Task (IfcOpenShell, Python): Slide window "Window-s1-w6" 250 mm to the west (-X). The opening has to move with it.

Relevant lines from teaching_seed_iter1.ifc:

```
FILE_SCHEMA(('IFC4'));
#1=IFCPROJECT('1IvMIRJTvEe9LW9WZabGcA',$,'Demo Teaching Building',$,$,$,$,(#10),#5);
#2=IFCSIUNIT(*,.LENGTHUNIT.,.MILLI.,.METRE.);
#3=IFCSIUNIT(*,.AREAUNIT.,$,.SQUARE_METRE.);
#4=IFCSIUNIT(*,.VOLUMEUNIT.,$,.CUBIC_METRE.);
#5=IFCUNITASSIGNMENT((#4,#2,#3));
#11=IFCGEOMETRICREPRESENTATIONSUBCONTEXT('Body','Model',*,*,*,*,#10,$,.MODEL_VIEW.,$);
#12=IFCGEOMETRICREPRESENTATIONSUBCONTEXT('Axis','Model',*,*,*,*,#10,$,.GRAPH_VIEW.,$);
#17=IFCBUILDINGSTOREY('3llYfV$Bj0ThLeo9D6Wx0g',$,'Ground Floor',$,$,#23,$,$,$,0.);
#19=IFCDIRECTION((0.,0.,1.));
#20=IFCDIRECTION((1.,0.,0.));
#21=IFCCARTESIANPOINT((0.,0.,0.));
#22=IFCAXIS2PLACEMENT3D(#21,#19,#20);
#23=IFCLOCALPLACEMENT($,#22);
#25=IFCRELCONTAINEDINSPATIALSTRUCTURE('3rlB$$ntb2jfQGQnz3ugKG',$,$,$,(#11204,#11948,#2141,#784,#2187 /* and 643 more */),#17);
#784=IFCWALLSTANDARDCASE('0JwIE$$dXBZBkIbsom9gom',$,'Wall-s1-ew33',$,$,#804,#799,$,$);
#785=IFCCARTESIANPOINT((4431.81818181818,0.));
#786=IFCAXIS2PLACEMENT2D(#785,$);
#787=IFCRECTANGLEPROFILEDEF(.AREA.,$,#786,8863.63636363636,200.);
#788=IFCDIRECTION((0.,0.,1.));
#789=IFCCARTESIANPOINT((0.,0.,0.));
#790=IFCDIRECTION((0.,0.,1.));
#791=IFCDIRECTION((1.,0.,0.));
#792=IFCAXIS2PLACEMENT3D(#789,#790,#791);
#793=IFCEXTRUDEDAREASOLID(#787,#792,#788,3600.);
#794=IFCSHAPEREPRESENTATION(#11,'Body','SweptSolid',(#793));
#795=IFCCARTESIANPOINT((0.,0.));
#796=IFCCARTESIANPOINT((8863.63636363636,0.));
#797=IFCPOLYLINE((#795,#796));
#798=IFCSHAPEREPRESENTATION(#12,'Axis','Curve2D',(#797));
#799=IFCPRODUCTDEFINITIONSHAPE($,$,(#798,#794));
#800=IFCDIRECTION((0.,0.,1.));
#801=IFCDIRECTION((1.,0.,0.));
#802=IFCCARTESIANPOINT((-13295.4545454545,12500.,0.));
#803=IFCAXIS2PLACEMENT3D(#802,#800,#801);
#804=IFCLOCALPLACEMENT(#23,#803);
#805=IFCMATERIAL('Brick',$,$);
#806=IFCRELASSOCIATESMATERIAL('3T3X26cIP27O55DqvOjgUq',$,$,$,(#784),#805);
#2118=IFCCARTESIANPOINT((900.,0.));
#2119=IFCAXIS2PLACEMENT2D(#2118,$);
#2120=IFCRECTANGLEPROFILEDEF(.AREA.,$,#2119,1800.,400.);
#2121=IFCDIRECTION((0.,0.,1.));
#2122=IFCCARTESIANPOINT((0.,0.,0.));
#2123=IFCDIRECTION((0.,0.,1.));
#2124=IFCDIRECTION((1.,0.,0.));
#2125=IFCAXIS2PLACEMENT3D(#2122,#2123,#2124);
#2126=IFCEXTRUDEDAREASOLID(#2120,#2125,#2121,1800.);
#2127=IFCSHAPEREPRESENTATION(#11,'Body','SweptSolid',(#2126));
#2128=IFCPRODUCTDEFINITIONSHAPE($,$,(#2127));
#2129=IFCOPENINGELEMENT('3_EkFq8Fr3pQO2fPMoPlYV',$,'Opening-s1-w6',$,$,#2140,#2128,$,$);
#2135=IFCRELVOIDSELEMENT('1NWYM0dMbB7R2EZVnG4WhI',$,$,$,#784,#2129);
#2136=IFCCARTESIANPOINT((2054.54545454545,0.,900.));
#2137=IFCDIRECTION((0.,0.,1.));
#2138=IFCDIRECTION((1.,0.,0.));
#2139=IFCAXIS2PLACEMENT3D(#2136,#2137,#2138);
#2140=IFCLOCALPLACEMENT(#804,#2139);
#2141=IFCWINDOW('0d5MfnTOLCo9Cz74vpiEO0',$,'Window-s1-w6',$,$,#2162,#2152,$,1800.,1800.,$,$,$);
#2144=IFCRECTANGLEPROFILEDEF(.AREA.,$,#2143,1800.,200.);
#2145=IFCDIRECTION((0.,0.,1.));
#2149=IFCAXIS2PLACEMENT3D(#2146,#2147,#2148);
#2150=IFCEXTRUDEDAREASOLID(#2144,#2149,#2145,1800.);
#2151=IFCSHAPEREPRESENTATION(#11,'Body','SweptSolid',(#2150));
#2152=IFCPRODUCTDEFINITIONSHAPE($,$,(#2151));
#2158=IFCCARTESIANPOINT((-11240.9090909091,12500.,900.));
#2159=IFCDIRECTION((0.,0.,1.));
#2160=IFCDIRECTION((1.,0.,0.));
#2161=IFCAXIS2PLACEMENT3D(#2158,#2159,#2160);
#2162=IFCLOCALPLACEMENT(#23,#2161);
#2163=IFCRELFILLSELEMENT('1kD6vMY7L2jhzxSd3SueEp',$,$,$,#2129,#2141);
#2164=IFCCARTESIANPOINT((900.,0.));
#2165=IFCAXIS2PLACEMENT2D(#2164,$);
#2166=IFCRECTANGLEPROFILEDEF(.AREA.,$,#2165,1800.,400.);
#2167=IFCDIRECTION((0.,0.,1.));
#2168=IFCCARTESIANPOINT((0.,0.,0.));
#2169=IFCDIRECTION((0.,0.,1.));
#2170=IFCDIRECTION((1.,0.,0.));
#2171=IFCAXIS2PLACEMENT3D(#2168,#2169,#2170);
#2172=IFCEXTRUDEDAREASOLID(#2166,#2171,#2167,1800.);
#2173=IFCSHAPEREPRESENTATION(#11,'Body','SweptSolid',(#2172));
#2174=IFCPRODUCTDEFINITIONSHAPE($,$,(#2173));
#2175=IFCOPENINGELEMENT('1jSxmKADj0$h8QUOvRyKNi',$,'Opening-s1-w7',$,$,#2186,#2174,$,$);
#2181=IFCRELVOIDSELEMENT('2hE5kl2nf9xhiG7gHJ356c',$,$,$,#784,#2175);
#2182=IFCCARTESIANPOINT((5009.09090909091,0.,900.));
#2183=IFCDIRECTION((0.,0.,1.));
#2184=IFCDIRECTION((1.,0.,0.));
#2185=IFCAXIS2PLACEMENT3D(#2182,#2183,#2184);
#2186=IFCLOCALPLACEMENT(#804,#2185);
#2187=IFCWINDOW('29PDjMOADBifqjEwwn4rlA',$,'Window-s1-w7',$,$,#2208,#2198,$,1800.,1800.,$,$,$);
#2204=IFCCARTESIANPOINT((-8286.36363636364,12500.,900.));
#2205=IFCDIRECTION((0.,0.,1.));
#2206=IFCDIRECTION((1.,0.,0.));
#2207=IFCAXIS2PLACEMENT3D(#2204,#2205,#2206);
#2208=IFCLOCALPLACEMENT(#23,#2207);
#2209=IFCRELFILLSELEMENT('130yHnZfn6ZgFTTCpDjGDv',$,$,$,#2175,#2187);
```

```python
import ifcopenshell
import ifcopenshell.api.geometry
import ifcopenshell.util.placement

model = ifcopenshell.open("teaching_seed_iter1.ifc")

window = model.by_guid("0d5MfnTOLCo9Cz74vpiEO0")
opening = window.FillsVoids[0].RelatingOpeningElement
wall = opening.VoidsElements[0].RelatingBuildingElement

wall_matrix = ifcopenshell.util.placement.get_local_placement(wall.ObjectPlacement)
shift = wall_matrix[:3, 0] * -250.0
before = ifcopenshell.util.placement.get_local_placement(window.ObjectPlacement)[:3, 3].copy()

# The window is not placed relative to its opening, so move both.
for product in (opening, window):
    matrix = ifcopenshell.util.placement.get_local_placement(product.ObjectPlacement)
    matrix[:3, 3] += shift
    ifcopenshell.api.geometry.edit_object_placement(model, product=product, matrix=matrix, is_si=False)

after = ifcopenshell.util.placement.get_local_placement(window.ObjectPlacement)[:3, 3]
print("window moved by", (after - before).round(3) + 0.0)

model.write("teaching_seed_iter1_v2.ifc")
```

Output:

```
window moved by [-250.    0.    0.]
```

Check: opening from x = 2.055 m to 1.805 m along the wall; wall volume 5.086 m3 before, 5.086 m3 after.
